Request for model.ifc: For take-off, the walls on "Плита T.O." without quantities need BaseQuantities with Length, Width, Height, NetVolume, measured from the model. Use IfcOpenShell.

First a look at what the model holds.

```python
import ifcopenshell
import ifcopenshell.util.element
import ifcopenshell.util.unit

model = ifcopenshell.open("model.ifc")
print(model.schema)
for unit_type in ("LENGTHUNIT", "AREAUNIT", "VOLUMEUNIT"):
    print(unit_type, ifcopenshell.util.unit.calculate_unit_scale(model, unit_type))
storey = next(s for s in model.by_type("IfcBuildingStorey") if s.Name == "Плита T.O.")
walls = [e for e in ifcopenshell.util.element.get_decomposition(storey) if e.is_a("IfcWall")]
for e in sorted(walls, key=lambda e: e.id()):
    print(e.id(), e.is_a(), e.Name, list(ifcopenshell.util.element.get_psets(e, qtos_only=True)), sep=" | ")
```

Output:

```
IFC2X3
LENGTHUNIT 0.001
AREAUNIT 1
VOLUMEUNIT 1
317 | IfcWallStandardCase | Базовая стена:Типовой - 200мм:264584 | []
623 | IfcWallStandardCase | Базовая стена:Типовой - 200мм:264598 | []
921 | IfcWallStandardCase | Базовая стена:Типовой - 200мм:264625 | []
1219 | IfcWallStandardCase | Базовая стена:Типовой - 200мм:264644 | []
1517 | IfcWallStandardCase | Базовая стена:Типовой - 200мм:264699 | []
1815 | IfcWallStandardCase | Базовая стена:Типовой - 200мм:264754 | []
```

```python
import ifcopenshell
import ifcopenshell.api.pset
import ifcopenshell.geom
import ifcopenshell.util.element
import ifcopenshell.util.shape
import ifcopenshell.util.unit

model = ifcopenshell.open("model.ifc")
unit_scale = ifcopenshell.util.unit.calculate_unit_scale(model)
volume_scale = ifcopenshell.util.unit.calculate_unit_scale(model, "VOLUMEUNIT")
settings = ifcopenshell.geom.settings()

storey = next(s for s in model.by_type("IfcBuildingStorey") if s.Name == "Плита T.O.")
walls = [e for e in ifcopenshell.util.element.get_decomposition(storey) if e.is_a("IfcWall")]

for e in sorted(walls, key=lambda e: e.id()):
    if ifcopenshell.util.element.get_psets(e, qtos_only=True, should_inherit=False):
        continue
    # Geometry comes back in metres, in the element's own axes.
    shape = ifcopenshell.geom.create_shape(settings, e)
    values = {
        "Length": ifcopenshell.util.shape.get_x(shape.geometry) / unit_scale,
        "Width": ifcopenshell.util.shape.get_y(shape.geometry) / unit_scale,
        "Height": ifcopenshell.util.shape.get_z(shape.geometry) / unit_scale,
        "NetVolume": ifcopenshell.util.shape.get_volume(shape.geometry) / volume_scale,
    }
    qto = ifcopenshell.api.pset.add_qto(model, product=e, name="BaseQuantities")
    ifcopenshell.api.pset.edit_qto(model, qto=qto, properties=values)
    print(e.id(), {k: round(v, 3) for k, v in values.items()})

model.write("model_rev.ifc")
```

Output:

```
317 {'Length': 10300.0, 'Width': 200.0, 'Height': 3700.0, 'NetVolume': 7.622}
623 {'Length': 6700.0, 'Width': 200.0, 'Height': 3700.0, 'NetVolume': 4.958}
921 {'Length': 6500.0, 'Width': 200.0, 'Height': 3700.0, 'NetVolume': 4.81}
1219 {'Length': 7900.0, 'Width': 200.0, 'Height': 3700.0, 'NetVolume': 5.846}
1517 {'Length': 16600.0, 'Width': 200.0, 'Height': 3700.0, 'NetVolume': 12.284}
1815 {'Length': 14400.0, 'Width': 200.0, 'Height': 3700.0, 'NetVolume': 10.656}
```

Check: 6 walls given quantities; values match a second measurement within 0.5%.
